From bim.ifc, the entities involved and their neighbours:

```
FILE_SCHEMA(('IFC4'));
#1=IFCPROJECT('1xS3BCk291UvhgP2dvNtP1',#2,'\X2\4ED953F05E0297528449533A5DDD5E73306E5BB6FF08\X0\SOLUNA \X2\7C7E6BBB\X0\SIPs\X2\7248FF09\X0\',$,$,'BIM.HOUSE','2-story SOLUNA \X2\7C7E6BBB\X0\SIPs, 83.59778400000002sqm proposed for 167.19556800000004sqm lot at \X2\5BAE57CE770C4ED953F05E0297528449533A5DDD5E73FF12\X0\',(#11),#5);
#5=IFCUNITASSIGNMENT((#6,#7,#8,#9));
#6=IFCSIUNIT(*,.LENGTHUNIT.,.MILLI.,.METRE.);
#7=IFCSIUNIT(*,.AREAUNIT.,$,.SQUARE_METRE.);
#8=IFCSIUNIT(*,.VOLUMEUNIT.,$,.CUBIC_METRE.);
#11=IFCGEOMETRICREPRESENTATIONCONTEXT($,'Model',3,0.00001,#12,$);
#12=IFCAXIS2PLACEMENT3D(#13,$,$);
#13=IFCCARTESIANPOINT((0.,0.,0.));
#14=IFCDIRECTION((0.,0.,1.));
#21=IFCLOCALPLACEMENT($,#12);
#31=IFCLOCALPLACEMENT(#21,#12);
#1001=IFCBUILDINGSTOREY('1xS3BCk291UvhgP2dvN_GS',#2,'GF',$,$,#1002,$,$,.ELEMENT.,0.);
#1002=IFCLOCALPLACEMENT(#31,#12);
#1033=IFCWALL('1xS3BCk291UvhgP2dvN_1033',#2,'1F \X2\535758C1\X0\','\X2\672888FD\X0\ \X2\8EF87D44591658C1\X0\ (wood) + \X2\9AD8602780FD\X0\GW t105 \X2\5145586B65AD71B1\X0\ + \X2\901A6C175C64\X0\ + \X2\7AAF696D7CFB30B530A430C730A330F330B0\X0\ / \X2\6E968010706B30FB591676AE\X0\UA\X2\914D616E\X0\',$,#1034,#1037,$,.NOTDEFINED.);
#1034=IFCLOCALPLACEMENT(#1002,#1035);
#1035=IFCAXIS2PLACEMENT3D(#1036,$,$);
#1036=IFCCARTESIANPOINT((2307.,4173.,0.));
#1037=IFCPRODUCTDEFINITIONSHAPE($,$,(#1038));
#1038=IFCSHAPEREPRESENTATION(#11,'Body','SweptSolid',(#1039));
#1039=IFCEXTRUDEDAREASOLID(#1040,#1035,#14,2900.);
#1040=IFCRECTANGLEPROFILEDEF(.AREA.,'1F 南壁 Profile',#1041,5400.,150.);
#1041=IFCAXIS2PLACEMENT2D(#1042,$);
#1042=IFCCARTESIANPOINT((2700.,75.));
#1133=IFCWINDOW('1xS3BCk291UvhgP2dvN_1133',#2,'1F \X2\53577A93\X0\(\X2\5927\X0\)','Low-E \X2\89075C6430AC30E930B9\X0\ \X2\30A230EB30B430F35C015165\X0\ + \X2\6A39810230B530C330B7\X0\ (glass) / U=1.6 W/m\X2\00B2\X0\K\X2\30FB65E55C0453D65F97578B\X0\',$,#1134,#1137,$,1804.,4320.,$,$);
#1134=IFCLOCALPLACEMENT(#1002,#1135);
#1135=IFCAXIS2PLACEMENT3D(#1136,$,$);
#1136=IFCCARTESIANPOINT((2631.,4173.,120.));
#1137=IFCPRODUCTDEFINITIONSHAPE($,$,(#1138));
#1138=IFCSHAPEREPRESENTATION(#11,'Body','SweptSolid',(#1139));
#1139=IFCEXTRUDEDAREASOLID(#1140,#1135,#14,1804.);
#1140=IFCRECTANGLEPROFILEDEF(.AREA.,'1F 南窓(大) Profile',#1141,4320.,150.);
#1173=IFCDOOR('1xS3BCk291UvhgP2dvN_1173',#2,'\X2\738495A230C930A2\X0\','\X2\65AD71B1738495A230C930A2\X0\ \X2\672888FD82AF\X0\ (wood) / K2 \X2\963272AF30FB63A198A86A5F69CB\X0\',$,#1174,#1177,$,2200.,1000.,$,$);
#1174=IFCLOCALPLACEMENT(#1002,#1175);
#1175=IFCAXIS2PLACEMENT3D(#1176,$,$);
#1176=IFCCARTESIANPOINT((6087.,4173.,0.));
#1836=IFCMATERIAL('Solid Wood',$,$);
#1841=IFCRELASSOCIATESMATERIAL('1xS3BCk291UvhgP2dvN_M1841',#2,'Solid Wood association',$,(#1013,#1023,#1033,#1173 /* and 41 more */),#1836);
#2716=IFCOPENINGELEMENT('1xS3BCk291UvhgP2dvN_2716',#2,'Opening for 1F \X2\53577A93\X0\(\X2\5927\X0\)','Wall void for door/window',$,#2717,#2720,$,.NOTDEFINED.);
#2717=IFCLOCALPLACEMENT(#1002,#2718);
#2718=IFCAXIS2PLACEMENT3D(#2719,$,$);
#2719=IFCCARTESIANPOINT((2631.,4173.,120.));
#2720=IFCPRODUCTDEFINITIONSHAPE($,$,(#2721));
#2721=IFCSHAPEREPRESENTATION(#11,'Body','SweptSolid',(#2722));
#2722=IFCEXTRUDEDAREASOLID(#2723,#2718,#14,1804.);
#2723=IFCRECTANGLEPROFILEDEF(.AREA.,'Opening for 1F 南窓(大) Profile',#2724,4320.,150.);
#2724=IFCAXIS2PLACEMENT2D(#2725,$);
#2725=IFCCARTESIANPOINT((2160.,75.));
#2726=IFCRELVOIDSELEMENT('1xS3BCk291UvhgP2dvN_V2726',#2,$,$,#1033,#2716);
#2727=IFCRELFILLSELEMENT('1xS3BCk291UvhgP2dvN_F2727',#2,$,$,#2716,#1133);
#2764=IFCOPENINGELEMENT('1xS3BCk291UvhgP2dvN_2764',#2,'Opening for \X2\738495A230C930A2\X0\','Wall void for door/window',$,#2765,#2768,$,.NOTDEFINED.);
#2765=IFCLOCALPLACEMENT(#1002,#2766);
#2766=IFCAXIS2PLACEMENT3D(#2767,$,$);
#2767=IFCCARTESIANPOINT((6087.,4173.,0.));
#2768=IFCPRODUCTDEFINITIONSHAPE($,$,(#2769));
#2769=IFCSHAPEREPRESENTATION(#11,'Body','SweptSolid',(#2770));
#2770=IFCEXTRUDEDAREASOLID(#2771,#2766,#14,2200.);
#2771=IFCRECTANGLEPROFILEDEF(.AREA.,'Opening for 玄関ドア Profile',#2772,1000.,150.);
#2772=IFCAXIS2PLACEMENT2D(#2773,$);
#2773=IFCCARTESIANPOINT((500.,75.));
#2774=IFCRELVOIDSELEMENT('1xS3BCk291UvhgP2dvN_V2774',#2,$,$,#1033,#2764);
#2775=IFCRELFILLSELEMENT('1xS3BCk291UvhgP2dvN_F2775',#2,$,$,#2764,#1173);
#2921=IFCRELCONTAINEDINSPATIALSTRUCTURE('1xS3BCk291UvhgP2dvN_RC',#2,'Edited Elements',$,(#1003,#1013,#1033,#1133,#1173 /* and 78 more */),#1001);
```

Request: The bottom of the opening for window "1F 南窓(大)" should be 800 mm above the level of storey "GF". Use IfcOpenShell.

```python
import numpy as np
import ifcopenshell
import ifcopenshell.api.geometry
import ifcopenshell.geom
import ifcopenshell.util.element
import ifcopenshell.util.placement
import ifcopenshell.util.shape
import ifcopenshell.util.unit

model = ifcopenshell.open("bim.ifc")
unit_scale = ifcopenshell.util.unit.calculate_unit_scale(model)

window = model.by_id(1133)
opening = window.FillsVoids[0].RelatingOpeningElement
storey = ifcopenshell.util.element.get_container(window, ifc_class="IfcBuildingStorey")
level = ifcopenshell.util.placement.get_local_placement(storey.ObjectPlacement)[2, 3]

# The opening's origin need not be at the sill, so measure its lowest point.
shape = ifcopenshell.geom.create_shape(ifcopenshell.geom.settings(), opening)
bottom = ifcopenshell.util.shape.get_shape_bottom_elevation(shape, shape.geometry) / unit_scale
dz = level + 0.8 / unit_scale - bottom

shift = np.array([0.0, 0.0, dz])
# The window is not placed relative to its opening, so move both.
for product in (opening, window):
    matrix = ifcopenshell.util.placement.get_local_placement(product.ObjectPlacement)
    matrix[:3, 3] += shift
    ifcopenshell.api.geometry.edit_object_placement(model, product=product, matrix=matrix, is_si=False)

print(f"moved by {dz * unit_scale:+.3f} m")

model.write("bim_updated.ifc")
```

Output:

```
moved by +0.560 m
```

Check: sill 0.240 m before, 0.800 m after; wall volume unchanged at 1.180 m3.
